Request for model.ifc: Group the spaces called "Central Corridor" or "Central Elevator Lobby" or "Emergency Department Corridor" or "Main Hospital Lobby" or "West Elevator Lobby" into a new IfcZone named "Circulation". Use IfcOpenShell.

First a look at what the model holds.

```python
import ifcopenshell

model = ifcopenshell.open("model.ifc")
print(model.schema)
seen = {}
for space in model.by_type("IfcSpace"):
    seen[space.Name] = seen.get(space.Name, 0) + 1
for name, count in sorted(seen.items(), key=str):
    print(count, "x", name)
print("zones:", [z.Name for z in model.by_type("IfcZone")][:20])
```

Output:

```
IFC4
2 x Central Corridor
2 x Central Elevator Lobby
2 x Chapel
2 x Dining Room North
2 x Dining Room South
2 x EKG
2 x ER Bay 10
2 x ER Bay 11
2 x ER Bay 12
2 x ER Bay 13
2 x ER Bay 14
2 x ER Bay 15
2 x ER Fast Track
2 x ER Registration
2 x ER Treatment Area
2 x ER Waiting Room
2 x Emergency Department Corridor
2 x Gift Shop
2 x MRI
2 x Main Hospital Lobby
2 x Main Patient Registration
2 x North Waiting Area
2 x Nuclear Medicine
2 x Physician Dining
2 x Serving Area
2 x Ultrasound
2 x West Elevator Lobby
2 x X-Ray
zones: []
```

```python
import ifcopenshell
import ifcopenshell.api.group
import ifcopenshell.api.root

model = ifcopenshell.open("model.ifc")

names = {"Central Corridor", "Central Elevator Lobby", "Emergency Department Corridor", "Main Hospital Lobby", "West Elevator Lobby"}
spaces = [s for s in model.by_type("IfcSpace") if s.Name in names]

zone = ifcopenshell.api.root.create_entity(model, ifc_class="IfcZone", name="Circulation")
ifcopenshell.api.group.assign_group(model, products=spaces, group=zone)
print(len(spaces), "spaces in", zone.Name)

model.write("model_v2.ifc")
```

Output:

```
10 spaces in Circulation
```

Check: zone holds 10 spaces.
